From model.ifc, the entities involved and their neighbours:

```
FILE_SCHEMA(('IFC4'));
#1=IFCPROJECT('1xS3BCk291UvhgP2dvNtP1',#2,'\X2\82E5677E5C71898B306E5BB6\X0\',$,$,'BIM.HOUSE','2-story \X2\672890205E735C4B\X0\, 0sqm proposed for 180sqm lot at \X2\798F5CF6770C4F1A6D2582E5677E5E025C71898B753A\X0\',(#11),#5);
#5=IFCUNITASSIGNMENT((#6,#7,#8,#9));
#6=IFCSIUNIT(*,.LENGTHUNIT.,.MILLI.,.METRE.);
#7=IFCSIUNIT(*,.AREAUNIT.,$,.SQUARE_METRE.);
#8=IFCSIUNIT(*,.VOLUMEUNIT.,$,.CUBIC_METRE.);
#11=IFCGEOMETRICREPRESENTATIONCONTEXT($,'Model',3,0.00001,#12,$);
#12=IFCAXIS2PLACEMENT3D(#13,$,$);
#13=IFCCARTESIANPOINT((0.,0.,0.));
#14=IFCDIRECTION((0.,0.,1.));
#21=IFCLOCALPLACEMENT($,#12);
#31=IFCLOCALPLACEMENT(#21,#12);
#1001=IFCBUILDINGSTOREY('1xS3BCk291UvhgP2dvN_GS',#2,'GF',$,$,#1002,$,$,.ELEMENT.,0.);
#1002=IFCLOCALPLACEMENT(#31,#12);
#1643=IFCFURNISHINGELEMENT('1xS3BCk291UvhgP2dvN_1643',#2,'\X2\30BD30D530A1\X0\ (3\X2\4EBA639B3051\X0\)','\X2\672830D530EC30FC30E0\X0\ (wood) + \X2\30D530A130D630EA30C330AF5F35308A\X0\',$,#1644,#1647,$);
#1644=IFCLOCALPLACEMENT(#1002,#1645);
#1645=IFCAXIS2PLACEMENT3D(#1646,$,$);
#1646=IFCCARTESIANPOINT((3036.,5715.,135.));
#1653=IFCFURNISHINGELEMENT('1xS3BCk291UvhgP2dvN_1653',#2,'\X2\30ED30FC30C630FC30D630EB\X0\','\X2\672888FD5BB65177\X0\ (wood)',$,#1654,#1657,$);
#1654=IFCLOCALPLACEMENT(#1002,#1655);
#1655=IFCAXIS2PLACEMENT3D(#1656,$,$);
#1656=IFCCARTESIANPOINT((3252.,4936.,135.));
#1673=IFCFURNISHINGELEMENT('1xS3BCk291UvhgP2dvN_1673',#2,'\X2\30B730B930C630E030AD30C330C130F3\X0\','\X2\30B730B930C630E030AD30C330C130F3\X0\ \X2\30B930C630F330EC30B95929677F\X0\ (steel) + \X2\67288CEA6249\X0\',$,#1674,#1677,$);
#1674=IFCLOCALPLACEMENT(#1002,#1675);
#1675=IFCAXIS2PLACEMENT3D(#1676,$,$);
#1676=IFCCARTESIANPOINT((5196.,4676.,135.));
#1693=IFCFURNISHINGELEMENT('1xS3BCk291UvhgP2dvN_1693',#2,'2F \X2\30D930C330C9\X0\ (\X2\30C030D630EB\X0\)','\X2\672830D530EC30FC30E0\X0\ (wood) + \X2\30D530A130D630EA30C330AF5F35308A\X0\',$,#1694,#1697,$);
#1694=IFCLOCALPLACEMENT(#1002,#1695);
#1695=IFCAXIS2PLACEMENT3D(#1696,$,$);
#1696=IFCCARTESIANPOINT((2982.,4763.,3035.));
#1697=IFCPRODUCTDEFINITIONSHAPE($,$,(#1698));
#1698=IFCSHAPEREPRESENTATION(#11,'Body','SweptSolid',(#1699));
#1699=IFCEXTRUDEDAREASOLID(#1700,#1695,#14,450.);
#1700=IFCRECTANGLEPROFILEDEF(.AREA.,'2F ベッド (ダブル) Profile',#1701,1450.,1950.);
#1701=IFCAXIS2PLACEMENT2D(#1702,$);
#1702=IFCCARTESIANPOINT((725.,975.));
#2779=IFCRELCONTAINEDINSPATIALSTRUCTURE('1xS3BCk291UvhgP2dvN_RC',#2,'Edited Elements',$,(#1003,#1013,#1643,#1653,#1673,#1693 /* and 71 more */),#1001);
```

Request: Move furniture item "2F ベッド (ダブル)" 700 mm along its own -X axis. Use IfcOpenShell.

```python
import ifcopenshell
import ifcopenshell.api.geometry
import ifcopenshell.util.placement
import ifcopenshell.util.unit

model = ifcopenshell.open("model.ifc")
unit_scale = ifcopenshell.util.unit.calculate_unit_scale(model)

item = model.by_id(1693)
matrix = ifcopenshell.util.placement.get_local_placement(item.ObjectPlacement)
matrix[:3, 3] -= matrix[:3, 0] * 0.7 / unit_scale
ifcopenshell.api.geometry.edit_object_placement(model, product=item, matrix=matrix, is_si=False)

print(ifcopenshell.util.placement.get_local_placement(item.ObjectPlacement).round(3) + 0.0)

model.write("model_rev.ifc")
```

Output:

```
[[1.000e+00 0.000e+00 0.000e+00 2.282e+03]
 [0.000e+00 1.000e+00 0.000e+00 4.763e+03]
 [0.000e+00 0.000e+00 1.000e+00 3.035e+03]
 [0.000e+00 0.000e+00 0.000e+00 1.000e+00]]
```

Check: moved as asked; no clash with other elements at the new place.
